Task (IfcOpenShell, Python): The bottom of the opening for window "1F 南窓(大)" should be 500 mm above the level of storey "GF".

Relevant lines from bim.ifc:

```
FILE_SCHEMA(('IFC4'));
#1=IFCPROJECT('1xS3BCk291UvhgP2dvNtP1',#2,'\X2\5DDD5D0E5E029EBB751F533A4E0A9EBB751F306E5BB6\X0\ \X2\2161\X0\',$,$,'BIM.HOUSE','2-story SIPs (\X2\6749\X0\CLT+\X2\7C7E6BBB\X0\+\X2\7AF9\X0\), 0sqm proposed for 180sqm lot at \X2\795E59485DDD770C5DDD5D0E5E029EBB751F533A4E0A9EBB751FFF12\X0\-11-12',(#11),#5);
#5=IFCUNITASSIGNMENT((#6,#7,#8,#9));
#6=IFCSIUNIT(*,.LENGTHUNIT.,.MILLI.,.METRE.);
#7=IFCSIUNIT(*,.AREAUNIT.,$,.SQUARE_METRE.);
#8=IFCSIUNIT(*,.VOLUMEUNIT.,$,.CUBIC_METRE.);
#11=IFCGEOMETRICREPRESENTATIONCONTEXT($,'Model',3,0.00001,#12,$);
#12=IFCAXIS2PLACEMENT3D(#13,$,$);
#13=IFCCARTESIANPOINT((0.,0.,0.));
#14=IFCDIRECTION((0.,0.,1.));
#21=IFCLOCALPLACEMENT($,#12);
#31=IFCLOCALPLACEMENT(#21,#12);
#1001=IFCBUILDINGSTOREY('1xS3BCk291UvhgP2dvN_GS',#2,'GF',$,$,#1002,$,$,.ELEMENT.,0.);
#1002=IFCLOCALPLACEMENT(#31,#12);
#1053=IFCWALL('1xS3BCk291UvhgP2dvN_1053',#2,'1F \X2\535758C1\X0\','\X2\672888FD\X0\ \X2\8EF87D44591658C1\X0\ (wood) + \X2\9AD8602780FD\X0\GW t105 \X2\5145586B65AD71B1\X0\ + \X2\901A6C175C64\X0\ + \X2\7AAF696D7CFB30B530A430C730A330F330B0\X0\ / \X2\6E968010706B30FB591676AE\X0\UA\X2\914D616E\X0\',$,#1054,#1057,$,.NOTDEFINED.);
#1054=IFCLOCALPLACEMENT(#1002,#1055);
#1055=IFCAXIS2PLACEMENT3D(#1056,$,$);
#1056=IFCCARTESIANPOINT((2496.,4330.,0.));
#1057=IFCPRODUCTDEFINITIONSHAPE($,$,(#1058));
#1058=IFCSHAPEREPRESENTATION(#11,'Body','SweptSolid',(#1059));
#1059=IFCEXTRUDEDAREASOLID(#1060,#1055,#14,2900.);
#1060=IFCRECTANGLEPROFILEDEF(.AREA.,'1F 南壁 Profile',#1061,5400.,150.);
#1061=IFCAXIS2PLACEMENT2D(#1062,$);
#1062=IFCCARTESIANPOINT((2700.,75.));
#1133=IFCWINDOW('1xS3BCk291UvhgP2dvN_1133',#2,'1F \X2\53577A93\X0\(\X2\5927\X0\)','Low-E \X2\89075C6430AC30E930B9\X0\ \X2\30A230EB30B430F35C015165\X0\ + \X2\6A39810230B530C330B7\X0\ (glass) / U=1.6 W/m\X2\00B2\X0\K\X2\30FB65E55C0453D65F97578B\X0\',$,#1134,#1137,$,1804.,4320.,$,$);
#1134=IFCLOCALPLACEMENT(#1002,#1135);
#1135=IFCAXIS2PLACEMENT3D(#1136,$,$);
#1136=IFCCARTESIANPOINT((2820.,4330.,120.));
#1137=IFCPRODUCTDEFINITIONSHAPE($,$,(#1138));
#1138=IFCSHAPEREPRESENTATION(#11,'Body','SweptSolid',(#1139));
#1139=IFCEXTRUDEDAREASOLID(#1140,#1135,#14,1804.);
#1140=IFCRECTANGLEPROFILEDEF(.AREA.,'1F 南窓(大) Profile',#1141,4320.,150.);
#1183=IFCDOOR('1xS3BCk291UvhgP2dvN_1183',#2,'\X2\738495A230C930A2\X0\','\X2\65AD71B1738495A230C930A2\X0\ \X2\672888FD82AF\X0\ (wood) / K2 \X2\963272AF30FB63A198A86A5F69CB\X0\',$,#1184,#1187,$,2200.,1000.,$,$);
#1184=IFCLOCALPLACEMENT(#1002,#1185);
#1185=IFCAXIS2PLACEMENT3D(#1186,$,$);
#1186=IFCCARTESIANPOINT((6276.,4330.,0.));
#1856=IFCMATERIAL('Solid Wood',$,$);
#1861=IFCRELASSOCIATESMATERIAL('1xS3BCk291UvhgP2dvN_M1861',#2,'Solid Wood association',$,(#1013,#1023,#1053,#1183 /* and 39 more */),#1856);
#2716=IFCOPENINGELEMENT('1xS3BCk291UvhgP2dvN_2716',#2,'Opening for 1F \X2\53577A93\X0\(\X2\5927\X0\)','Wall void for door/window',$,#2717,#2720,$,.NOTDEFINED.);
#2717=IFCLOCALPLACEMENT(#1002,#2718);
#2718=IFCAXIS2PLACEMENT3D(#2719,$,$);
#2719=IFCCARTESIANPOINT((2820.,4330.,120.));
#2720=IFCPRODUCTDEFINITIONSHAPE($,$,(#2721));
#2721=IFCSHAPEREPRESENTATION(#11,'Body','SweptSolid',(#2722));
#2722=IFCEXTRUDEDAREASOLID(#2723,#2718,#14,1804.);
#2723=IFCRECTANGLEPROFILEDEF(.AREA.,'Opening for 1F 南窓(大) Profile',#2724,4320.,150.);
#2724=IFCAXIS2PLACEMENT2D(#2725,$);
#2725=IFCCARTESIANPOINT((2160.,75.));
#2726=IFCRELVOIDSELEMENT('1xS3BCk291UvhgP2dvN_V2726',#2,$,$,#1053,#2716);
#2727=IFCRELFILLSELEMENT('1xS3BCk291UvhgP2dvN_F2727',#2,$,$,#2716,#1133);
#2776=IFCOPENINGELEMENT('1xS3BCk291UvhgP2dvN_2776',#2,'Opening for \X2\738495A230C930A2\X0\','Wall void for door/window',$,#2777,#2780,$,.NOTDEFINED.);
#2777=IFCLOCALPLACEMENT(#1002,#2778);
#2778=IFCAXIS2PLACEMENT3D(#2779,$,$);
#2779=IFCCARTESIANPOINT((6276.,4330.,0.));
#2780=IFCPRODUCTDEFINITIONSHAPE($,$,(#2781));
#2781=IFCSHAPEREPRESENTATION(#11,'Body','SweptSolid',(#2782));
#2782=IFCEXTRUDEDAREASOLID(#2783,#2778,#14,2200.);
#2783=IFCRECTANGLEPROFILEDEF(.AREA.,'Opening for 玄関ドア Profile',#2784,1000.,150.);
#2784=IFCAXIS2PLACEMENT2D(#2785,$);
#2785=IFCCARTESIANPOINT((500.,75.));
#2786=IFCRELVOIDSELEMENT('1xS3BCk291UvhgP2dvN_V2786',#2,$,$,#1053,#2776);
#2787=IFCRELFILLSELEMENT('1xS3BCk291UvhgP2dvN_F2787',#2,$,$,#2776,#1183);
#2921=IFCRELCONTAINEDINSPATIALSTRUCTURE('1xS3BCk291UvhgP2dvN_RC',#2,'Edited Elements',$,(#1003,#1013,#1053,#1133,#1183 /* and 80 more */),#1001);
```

```python
import numpy as np
import ifcopenshell
import ifcopenshell.api.geometry
import ifcopenshell.geom
import ifcopenshell.util.element
import ifcopenshell.util.placement
import ifcopenshell.util.shape
import ifcopenshell.util.unit

model = ifcopenshell.open("bim.ifc")
unit_scale = ifcopenshell.util.unit.calculate_unit_scale(model)

window = model.by_id(1133)
opening = window.FillsVoids[0].RelatingOpeningElement
storey = ifcopenshell.util.element.get_container(window, ifc_class="IfcBuildingStorey")
level = ifcopenshell.util.placement.get_local_placement(storey.ObjectPlacement)[2, 3]

# The opening's origin need not be at the sill, so measure its lowest point.
shape = ifcopenshell.geom.create_shape(ifcopenshell.geom.settings(), opening)
bottom = ifcopenshell.util.shape.get_shape_bottom_elevation(shape, shape.geometry) / unit_scale
dz = level + 500.0 - bottom

shift = np.array([0.0, 0.0, dz])
# The window is not placed relative to its opening, so move both.
for product in (opening, window):
    matrix = ifcopenshell.util.placement.get_local_placement(product.ObjectPlacement)
    matrix[:3, 3] += shift
    ifcopenshell.api.geometry.edit_object_placement(model, product=product, matrix=matrix, is_si=False)

print(f"moved by {dz * unit_scale:+.3f} m")

model.write("bim-out.ifc")
```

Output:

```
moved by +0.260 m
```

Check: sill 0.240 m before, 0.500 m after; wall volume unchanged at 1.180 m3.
